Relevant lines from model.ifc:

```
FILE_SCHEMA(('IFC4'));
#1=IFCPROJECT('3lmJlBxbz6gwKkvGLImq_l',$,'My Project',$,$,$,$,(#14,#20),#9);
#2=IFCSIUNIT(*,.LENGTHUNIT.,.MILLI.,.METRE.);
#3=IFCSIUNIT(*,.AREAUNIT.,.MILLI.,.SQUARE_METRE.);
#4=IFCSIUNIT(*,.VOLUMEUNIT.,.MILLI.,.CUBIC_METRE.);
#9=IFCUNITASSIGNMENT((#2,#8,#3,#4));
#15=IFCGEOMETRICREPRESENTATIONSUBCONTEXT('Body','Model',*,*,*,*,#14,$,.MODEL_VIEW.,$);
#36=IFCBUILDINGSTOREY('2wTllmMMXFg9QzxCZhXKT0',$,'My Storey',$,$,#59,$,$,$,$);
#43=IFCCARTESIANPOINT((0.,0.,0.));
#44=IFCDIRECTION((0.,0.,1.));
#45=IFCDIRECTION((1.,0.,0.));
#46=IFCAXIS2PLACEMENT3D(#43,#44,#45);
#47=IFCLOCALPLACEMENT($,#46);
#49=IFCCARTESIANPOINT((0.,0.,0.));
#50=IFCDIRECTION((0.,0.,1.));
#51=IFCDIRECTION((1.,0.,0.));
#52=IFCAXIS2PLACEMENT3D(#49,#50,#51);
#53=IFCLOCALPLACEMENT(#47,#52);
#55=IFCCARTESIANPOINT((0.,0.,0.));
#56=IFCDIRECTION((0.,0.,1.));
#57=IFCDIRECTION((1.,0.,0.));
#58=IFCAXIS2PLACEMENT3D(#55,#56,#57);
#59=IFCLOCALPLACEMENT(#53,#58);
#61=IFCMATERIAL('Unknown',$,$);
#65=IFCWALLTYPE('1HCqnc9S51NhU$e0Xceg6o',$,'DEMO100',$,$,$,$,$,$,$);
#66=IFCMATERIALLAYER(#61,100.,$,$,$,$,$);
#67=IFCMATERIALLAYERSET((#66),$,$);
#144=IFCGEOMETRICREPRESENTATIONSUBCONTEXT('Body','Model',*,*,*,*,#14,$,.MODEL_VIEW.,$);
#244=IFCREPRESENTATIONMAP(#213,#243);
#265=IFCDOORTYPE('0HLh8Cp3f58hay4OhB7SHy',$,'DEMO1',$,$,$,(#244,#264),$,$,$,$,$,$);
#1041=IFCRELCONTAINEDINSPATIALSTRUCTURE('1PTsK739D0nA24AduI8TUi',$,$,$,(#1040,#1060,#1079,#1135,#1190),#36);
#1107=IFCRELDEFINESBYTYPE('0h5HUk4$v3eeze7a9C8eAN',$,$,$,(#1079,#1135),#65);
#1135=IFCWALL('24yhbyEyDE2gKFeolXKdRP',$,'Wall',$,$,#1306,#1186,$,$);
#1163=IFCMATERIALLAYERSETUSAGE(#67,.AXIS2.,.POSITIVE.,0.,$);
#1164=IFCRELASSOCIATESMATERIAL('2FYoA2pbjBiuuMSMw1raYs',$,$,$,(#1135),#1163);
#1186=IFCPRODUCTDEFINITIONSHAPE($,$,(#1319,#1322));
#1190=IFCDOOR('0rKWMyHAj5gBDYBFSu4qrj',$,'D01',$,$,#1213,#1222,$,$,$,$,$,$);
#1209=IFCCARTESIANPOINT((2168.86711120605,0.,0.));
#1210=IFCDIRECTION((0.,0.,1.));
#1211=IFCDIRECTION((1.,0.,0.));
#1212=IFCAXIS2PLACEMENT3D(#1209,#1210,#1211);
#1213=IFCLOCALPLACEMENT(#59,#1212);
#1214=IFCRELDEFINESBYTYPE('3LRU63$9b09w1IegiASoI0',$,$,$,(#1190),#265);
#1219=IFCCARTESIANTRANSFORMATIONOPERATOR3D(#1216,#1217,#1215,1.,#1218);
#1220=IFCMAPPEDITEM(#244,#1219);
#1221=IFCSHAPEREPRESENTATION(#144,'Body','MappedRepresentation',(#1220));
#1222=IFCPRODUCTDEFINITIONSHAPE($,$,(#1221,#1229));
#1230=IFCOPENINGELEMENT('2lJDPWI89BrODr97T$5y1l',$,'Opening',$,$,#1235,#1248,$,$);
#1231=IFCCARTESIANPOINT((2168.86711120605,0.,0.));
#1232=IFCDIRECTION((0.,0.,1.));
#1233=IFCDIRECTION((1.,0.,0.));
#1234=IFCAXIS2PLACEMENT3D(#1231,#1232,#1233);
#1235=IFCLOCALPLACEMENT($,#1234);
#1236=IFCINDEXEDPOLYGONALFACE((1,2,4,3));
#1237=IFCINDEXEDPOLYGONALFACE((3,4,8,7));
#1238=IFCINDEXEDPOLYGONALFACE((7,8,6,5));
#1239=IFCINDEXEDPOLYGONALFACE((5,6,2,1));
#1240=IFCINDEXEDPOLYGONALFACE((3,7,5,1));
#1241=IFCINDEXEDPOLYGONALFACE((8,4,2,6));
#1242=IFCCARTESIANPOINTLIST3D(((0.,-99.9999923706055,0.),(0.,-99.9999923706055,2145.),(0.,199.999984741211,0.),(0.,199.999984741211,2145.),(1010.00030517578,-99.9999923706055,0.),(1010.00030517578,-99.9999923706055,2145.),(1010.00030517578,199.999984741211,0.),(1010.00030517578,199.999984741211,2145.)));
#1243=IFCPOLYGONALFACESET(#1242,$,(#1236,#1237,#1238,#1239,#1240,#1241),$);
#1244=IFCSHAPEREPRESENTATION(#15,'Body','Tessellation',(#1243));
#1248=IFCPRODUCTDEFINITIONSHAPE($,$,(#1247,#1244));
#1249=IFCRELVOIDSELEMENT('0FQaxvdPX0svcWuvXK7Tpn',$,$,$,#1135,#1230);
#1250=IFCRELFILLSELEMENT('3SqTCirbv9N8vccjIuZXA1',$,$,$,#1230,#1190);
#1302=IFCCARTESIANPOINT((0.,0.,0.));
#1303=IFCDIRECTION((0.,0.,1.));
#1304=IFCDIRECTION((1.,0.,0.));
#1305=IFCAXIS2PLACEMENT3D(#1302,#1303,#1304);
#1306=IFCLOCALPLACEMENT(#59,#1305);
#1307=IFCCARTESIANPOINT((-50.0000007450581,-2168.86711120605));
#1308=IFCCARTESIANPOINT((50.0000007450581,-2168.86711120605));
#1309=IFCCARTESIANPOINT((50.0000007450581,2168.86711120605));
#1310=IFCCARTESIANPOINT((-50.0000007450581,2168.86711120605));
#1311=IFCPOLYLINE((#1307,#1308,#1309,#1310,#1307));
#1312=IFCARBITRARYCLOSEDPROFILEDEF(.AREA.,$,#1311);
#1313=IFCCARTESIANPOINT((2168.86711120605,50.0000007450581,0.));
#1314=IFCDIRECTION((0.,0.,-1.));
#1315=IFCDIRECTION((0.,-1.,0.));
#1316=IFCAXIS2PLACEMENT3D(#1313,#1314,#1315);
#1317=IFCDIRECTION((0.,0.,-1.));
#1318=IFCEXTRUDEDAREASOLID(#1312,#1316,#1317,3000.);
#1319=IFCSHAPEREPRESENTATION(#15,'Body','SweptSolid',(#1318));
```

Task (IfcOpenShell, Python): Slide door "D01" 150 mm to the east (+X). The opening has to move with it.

```python
import ifcopenshell
import ifcopenshell.api.geometry
import ifcopenshell.util.placement

model = ifcopenshell.open("model.ifc")

door = model.by_guid("0rKWMyHAj5gBDYBFSu4qrj")
opening = door.FillsVoids[0].RelatingOpeningElement
wall = opening.VoidsElements[0].RelatingBuildingElement

wall_matrix = ifcopenshell.util.placement.get_local_placement(wall.ObjectPlacement)
shift = wall_matrix[:3, 0] * 150.0
before = ifcopenshell.util.placement.get_local_placement(door.ObjectPlacement)[:3, 3].copy()

# The door is not placed relative to its opening, so move both.
for product in (opening, door):
    matrix = ifcopenshell.util.placement.get_local_placement(product.ObjectPlacement)
    matrix[:3, 3] += shift
    ifcopenshell.api.geometry.edit_object_placement(model, product=product, matrix=matrix, is_si=False)

after = ifcopenshell.util.placement.get_local_placement(door.ObjectPlacement)[:3, 3]
print("door moved by", (after - before).round(3) + 0.0)

model.write("model_rev.ifc")
```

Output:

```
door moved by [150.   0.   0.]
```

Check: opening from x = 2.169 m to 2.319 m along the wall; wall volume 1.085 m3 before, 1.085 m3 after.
